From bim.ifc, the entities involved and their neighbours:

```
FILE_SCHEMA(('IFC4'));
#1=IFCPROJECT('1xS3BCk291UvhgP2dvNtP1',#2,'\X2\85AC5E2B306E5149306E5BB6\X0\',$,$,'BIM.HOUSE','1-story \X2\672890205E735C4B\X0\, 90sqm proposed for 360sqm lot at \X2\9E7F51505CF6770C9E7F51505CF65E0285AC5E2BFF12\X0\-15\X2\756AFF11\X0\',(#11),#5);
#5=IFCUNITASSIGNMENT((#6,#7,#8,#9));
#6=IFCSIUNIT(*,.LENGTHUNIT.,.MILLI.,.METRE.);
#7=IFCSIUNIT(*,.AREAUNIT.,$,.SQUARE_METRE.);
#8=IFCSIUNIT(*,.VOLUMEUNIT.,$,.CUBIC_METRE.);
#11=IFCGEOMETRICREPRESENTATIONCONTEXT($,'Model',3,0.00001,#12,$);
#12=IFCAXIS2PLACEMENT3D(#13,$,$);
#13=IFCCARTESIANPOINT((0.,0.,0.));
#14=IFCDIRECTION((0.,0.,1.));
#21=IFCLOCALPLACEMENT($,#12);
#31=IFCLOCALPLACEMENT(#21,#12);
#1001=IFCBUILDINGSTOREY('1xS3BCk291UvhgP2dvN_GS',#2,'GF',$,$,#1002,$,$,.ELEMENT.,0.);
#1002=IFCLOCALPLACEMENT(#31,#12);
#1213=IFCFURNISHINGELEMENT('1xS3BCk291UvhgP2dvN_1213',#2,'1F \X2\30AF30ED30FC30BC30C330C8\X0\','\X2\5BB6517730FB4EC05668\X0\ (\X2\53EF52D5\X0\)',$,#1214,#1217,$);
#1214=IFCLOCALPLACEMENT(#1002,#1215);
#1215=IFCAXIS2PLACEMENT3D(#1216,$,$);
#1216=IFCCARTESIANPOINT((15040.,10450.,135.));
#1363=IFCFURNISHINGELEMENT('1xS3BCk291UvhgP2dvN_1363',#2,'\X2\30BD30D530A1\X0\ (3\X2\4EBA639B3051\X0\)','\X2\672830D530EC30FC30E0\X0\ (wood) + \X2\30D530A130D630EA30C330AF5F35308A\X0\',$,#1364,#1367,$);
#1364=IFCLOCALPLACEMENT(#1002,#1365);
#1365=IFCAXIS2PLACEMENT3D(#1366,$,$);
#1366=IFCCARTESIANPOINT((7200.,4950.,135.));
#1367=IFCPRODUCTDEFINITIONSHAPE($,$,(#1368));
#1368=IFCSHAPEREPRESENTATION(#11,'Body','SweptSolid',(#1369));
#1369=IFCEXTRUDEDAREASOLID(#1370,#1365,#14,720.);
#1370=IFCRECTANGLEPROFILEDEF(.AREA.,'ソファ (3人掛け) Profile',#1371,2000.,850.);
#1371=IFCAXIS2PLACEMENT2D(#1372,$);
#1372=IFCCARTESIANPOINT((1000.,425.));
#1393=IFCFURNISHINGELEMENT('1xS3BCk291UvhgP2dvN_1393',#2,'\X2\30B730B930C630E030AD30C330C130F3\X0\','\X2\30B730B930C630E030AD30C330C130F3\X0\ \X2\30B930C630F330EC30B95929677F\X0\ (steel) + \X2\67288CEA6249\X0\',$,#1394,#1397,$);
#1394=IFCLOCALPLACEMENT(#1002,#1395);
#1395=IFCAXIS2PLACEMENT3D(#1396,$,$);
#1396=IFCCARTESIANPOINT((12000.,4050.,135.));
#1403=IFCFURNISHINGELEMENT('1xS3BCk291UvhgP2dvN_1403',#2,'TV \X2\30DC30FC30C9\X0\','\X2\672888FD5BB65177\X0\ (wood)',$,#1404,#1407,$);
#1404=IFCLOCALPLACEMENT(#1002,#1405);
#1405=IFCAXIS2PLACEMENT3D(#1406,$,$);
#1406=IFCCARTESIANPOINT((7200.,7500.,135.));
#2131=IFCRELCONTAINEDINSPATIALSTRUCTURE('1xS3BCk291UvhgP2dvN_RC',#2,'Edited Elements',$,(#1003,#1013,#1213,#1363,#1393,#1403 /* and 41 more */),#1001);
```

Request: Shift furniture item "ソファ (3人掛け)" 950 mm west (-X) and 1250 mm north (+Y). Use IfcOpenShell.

```python
import ifcopenshell
import ifcopenshell.api.geometry
import ifcopenshell.util.placement
import ifcopenshell.util.unit

model = ifcopenshell.open("bim.ifc")
unit_scale = ifcopenshell.util.unit.calculate_unit_scale(model)

item = model.by_guid("1xS3BCk291UvhgP2dvN_1363")
matrix = ifcopenshell.util.placement.get_local_placement(item.ObjectPlacement)
matrix[0, 3] -= 0.95 / unit_scale
matrix[1, 3] += 1.25 / unit_scale
ifcopenshell.api.geometry.edit_object_placement(model, product=item, matrix=matrix, is_si=False)

print(ifcopenshell.util.placement.get_local_placement(item.ObjectPlacement).round(3) + 0.0)

model.write("bim_v2.ifc")
```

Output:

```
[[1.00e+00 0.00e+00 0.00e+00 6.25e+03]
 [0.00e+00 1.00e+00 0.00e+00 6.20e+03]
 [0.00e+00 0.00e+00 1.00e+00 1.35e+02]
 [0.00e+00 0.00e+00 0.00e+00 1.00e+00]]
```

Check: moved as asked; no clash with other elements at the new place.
